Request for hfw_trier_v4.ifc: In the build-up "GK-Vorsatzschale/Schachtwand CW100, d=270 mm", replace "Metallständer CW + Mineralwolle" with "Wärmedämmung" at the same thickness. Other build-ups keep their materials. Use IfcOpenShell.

First a look at what the model holds.

```python
import ifcopenshell
import ifcopenshell.util.element

model = ifcopenshell.open("hfw_trier_v4.ifc")
print(model.schema)
for layer_set in model.by_type("IfcMaterialLayerSet"):
    if layer_set.LayerSetName == "GK-Vorsatzschale/Schachtwand CW100, d=270 mm":
        for layer in layer_set.MaterialLayers:
            print(layer.id(), layer.Material and layer.Material.Name, layer.LayerThickness, sep=" | ")
        print(len(ifcopenshell.util.element.get_elements_by_material(model, layer_set)), "elements and types use it")
print(sorted(m.Name for m in model.by_type("IfcMaterial") if m.Name)[:60])
```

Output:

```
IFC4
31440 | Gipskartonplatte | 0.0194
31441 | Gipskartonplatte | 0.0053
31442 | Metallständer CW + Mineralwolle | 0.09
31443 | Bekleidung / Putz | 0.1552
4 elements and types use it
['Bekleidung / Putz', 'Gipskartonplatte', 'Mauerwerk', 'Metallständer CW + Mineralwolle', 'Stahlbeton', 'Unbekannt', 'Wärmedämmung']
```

```python
import ifcopenshell
import ifcopenshell.api.material

model = ifcopenshell.open("hfw_trier_v4.ifc")

layer_set = next(s for s in model.by_type("IfcMaterialLayerSet") if s.LayerSetName == "GK-Vorsatzschale/Schachtwand CW100, d=270 mm")
layer = next(l for l in layer_set.MaterialLayers if l.Material and l.Material.Name == "Metallständer CW + Mineralwolle")
material = next(m for m in model.by_type("IfcMaterial") if m.Name == "Wärmedämmung")

# Point this one layer at the other material; renaming the old one would change it everywhere.
ifcopenshell.api.material.edit_layer(model, layer=layer, attributes={"Name": material.Name}, material=material)

print([l.Material.Name if l.Material else None for l in layer_set.MaterialLayers])

model.write("hfw_trier_v4_rev.ifc")
```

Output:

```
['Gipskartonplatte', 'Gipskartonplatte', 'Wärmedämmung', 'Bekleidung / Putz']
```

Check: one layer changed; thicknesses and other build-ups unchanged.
